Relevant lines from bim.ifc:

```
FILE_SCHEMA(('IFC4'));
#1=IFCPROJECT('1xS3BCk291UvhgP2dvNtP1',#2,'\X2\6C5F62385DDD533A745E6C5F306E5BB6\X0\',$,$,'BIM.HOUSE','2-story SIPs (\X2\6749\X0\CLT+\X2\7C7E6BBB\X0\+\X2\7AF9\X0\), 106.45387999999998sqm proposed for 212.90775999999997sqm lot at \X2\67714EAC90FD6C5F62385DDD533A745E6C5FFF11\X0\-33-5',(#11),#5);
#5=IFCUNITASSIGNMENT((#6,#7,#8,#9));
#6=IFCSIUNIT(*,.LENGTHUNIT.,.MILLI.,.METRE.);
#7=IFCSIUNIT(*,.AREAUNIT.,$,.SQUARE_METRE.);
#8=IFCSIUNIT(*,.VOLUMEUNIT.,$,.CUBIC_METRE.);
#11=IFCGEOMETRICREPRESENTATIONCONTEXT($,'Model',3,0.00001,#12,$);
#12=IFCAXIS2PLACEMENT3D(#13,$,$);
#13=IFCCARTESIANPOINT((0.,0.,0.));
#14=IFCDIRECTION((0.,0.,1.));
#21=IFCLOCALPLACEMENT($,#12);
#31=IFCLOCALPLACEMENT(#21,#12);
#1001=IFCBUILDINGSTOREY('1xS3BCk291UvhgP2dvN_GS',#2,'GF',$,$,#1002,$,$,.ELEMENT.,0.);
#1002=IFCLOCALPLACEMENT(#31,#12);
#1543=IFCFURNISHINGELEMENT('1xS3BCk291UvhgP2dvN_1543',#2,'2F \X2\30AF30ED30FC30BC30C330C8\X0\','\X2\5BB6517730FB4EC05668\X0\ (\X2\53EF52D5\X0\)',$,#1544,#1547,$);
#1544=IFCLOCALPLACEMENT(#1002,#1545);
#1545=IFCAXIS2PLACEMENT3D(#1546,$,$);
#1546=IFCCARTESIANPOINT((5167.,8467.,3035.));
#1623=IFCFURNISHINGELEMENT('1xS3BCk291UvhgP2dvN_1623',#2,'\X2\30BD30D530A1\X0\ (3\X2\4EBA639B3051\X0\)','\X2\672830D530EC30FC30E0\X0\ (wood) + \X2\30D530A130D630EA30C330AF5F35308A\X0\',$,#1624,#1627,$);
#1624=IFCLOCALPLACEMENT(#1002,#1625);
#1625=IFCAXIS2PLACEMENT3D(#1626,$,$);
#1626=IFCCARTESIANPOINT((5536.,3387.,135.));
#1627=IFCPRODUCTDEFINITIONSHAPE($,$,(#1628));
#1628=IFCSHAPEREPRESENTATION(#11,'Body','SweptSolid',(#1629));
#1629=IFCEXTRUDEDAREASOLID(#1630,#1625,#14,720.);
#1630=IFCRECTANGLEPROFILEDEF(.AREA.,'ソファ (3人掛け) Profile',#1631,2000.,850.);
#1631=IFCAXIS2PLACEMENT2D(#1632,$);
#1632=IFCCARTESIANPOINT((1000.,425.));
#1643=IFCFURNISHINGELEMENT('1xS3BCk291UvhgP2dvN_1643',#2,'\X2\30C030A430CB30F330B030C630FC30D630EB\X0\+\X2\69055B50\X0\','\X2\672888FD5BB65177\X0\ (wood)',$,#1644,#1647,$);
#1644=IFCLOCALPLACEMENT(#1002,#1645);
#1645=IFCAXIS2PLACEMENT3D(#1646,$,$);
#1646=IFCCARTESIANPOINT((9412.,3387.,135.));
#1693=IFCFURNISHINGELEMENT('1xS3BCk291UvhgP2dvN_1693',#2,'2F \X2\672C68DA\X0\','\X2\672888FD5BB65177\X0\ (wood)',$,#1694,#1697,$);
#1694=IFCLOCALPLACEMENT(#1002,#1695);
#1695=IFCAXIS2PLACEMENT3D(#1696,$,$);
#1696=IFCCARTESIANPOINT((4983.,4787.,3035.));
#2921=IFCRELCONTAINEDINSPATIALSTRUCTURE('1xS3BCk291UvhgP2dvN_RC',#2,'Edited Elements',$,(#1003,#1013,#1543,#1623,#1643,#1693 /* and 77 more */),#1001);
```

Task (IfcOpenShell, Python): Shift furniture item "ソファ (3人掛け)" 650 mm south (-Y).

```python
import ifcopenshell
import ifcopenshell.api.geometry
import ifcopenshell.util.placement

model = ifcopenshell.open("bim.ifc")

item = model.by_guid("1xS3BCk291UvhgP2dvN_1623")
matrix = ifcopenshell.util.placement.get_local_placement(item.ObjectPlacement)
matrix[1, 3] -= 650.0
ifcopenshell.api.geometry.edit_object_placement(model, product=item, matrix=matrix, is_si=False)

print(ifcopenshell.util.placement.get_local_placement(item.ObjectPlacement).round(3) + 0.0)

model.write("bim_updated.ifc")
```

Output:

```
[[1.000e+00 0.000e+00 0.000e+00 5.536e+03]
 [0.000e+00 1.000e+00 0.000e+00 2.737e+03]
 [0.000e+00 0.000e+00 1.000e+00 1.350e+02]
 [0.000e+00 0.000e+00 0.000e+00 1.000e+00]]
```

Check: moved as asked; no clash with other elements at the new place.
